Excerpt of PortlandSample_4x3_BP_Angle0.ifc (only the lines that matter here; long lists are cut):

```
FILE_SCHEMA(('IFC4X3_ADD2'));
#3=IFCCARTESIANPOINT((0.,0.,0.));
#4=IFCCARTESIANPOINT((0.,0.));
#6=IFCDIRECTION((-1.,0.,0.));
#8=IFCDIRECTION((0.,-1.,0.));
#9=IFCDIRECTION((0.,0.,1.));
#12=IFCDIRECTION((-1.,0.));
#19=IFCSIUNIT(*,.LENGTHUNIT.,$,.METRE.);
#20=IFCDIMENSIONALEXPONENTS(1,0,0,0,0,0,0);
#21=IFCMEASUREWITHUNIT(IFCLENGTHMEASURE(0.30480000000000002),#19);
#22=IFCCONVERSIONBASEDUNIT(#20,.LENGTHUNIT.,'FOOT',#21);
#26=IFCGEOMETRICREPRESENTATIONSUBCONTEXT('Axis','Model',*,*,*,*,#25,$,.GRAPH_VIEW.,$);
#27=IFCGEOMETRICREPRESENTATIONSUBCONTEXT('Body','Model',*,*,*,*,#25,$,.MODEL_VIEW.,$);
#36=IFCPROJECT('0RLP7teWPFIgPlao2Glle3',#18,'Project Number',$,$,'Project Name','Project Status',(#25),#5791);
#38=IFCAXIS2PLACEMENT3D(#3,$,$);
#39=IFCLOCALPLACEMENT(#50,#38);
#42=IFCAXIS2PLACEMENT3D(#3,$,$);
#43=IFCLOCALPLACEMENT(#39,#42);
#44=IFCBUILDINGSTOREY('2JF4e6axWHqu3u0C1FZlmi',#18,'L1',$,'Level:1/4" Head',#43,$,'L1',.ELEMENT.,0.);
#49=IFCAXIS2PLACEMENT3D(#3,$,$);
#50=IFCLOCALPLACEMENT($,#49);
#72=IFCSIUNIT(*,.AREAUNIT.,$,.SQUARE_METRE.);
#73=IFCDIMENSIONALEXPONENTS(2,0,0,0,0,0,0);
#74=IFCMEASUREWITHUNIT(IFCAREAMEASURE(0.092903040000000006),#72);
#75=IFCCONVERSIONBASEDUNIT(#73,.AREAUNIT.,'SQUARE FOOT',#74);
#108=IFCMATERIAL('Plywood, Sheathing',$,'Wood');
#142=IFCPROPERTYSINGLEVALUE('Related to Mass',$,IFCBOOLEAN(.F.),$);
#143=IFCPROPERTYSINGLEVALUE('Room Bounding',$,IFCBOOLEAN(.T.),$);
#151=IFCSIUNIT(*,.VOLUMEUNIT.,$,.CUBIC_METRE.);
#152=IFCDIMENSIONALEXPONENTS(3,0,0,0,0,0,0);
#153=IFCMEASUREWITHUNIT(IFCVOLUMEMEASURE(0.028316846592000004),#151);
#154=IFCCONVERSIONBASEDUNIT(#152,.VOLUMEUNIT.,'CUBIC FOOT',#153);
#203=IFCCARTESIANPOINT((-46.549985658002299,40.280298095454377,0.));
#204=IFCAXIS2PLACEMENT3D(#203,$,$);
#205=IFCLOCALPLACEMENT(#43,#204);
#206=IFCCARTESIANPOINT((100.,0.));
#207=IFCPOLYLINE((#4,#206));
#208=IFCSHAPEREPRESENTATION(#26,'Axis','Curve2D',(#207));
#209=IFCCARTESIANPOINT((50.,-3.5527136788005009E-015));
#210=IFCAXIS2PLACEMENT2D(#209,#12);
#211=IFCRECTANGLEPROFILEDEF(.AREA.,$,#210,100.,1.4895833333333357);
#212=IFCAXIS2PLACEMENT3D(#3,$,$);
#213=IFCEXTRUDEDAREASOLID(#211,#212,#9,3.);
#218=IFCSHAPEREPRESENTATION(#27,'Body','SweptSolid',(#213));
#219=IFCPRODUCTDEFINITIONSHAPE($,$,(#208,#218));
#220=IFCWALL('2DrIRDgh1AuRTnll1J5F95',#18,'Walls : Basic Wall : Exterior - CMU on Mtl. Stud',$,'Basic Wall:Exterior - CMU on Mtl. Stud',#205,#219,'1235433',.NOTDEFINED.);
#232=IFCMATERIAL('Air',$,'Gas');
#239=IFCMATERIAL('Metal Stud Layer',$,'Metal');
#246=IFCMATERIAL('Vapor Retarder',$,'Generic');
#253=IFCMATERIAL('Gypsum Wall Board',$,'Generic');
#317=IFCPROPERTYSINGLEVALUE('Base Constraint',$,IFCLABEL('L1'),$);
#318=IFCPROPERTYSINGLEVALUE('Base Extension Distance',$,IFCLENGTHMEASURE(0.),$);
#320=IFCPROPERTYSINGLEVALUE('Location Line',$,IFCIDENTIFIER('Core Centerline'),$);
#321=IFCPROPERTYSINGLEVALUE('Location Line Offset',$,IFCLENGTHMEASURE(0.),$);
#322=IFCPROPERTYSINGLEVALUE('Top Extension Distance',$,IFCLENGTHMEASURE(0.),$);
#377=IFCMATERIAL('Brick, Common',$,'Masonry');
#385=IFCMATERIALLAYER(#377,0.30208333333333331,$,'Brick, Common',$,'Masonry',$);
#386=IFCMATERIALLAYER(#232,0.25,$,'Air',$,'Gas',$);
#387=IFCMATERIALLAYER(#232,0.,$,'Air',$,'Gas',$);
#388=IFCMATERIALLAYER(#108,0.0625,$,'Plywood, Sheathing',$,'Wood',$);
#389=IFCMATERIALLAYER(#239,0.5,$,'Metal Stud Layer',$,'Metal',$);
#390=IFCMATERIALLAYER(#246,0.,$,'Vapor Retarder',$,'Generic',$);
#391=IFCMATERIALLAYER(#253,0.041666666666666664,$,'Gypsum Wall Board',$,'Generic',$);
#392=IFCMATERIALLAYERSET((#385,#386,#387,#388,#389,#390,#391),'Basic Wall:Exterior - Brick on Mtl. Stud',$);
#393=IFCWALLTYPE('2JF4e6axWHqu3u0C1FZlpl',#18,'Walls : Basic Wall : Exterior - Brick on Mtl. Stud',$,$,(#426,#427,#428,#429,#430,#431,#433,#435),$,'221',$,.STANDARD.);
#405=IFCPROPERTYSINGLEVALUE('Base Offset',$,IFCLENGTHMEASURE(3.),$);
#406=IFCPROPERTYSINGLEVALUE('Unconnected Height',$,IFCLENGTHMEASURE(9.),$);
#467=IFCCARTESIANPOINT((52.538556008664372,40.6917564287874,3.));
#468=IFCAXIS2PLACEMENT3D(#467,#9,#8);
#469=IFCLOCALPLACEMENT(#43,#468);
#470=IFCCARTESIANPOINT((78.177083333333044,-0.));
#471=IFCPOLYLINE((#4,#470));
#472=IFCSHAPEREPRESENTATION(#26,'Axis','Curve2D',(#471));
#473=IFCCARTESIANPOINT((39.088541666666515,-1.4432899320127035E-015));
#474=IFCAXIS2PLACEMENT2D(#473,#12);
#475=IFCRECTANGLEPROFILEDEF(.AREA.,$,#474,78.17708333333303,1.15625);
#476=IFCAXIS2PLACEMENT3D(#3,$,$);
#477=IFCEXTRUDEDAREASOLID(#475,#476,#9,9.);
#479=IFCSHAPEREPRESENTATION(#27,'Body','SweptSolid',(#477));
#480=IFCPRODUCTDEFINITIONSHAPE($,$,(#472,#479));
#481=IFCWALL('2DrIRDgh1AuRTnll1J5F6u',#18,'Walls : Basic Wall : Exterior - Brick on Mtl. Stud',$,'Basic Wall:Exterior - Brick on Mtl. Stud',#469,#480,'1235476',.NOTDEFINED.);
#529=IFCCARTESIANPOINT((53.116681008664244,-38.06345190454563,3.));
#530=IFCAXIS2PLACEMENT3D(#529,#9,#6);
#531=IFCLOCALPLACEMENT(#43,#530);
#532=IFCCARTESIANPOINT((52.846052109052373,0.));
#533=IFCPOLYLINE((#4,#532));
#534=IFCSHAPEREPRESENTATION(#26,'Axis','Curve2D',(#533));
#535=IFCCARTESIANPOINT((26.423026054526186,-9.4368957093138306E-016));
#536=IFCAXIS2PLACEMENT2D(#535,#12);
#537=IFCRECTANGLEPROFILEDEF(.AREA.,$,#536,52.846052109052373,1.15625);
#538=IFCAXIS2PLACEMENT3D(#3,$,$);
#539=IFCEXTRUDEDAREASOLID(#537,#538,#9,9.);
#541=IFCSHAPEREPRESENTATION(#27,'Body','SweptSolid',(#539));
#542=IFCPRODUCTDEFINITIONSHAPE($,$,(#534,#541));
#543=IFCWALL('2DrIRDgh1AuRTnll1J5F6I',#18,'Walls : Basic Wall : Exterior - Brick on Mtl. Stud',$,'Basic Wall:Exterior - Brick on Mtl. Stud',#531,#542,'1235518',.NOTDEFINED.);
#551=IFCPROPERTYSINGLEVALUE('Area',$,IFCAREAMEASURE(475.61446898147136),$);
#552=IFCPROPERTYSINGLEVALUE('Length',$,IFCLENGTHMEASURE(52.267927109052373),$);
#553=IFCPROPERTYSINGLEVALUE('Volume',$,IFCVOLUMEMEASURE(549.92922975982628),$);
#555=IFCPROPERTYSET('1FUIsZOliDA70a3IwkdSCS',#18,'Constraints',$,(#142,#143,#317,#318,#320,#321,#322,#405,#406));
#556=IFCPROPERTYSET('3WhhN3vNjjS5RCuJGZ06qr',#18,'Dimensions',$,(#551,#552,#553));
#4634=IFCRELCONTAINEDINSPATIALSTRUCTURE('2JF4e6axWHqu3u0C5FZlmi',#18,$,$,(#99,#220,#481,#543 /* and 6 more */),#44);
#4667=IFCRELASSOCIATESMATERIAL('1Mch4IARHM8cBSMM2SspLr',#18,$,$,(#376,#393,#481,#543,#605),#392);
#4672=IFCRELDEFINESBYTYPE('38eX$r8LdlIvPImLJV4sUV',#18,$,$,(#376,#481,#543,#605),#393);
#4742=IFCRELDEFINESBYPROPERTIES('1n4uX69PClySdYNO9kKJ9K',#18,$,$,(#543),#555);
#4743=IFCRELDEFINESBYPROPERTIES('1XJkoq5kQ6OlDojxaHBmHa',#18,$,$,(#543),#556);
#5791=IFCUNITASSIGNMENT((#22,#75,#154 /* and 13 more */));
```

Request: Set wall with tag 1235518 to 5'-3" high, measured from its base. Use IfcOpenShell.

```python
import ifcopenshell
import ifcopenshell.api.pset
import ifcopenshell.geom
import ifcopenshell.util.element
import ifcopenshell.util.representation
import ifcopenshell.util.shape
import ifcopenshell.util.unit

model = ifcopenshell.open("PortlandSample_4x3_BP_Angle0.ifc")
unit_scale = ifcopenshell.util.unit.calculate_unit_scale(model)
area_scale = ifcopenshell.util.unit.calculate_unit_scale(model, "AREAUNIT")
volume_scale = ifcopenshell.util.unit.calculate_unit_scale(model, "VOLUMEUNIT")
settings = ifcopenshell.geom.settings()


def volume(element):
    """Net volume in cubic metres, openings subtracted."""
    shape = ifcopenshell.geom.create_shape(settings, element)
    return ifcopenshell.util.shape.get_volume(shape.geometry)


wall = model.by_id(543)
before = volume(wall)

body = ifcopenshell.util.representation.get_representation(wall, "Model", "Body")
solid = body.Items[0]
old_height = solid.Depth
solid.Depth = 63 * 0.0254 / unit_scale
after = volume(wall)
thickness = 0.3524  # wall thickness in metres

# Update the stored height, areas and volumes.
pset = model.by_id(ifcopenshell.util.element.get_pset(wall, "Constraints", should_inherit=False)["id"])
ifcopenshell.api.pset.edit_pset(model, pset=pset, properties={
    "Unconnected Height": model.create_entity("IfcLengthMeasure", solid.Depth),
})
pset = model.by_id(ifcopenshell.util.element.get_pset(wall, "Dimensions", should_inherit=False)["id"])
ifcopenshell.api.pset.edit_pset(model, pset=pset, properties={
    "Area": model.create_entity("IfcAreaMeasure", after / thickness / area_scale),
    "Volume": model.create_entity("IfcVolumeMeasure", after / volume_scale),
})

print(f"height {old_height:g} -> {solid.Depth:g}, volume {before:.3f} -> {after:.3f} m3")

model.write("PortlandSample_4x3_BP_Angle0_updated.ifc")
```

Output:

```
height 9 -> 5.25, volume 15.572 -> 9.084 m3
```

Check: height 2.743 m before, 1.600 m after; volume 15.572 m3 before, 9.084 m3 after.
